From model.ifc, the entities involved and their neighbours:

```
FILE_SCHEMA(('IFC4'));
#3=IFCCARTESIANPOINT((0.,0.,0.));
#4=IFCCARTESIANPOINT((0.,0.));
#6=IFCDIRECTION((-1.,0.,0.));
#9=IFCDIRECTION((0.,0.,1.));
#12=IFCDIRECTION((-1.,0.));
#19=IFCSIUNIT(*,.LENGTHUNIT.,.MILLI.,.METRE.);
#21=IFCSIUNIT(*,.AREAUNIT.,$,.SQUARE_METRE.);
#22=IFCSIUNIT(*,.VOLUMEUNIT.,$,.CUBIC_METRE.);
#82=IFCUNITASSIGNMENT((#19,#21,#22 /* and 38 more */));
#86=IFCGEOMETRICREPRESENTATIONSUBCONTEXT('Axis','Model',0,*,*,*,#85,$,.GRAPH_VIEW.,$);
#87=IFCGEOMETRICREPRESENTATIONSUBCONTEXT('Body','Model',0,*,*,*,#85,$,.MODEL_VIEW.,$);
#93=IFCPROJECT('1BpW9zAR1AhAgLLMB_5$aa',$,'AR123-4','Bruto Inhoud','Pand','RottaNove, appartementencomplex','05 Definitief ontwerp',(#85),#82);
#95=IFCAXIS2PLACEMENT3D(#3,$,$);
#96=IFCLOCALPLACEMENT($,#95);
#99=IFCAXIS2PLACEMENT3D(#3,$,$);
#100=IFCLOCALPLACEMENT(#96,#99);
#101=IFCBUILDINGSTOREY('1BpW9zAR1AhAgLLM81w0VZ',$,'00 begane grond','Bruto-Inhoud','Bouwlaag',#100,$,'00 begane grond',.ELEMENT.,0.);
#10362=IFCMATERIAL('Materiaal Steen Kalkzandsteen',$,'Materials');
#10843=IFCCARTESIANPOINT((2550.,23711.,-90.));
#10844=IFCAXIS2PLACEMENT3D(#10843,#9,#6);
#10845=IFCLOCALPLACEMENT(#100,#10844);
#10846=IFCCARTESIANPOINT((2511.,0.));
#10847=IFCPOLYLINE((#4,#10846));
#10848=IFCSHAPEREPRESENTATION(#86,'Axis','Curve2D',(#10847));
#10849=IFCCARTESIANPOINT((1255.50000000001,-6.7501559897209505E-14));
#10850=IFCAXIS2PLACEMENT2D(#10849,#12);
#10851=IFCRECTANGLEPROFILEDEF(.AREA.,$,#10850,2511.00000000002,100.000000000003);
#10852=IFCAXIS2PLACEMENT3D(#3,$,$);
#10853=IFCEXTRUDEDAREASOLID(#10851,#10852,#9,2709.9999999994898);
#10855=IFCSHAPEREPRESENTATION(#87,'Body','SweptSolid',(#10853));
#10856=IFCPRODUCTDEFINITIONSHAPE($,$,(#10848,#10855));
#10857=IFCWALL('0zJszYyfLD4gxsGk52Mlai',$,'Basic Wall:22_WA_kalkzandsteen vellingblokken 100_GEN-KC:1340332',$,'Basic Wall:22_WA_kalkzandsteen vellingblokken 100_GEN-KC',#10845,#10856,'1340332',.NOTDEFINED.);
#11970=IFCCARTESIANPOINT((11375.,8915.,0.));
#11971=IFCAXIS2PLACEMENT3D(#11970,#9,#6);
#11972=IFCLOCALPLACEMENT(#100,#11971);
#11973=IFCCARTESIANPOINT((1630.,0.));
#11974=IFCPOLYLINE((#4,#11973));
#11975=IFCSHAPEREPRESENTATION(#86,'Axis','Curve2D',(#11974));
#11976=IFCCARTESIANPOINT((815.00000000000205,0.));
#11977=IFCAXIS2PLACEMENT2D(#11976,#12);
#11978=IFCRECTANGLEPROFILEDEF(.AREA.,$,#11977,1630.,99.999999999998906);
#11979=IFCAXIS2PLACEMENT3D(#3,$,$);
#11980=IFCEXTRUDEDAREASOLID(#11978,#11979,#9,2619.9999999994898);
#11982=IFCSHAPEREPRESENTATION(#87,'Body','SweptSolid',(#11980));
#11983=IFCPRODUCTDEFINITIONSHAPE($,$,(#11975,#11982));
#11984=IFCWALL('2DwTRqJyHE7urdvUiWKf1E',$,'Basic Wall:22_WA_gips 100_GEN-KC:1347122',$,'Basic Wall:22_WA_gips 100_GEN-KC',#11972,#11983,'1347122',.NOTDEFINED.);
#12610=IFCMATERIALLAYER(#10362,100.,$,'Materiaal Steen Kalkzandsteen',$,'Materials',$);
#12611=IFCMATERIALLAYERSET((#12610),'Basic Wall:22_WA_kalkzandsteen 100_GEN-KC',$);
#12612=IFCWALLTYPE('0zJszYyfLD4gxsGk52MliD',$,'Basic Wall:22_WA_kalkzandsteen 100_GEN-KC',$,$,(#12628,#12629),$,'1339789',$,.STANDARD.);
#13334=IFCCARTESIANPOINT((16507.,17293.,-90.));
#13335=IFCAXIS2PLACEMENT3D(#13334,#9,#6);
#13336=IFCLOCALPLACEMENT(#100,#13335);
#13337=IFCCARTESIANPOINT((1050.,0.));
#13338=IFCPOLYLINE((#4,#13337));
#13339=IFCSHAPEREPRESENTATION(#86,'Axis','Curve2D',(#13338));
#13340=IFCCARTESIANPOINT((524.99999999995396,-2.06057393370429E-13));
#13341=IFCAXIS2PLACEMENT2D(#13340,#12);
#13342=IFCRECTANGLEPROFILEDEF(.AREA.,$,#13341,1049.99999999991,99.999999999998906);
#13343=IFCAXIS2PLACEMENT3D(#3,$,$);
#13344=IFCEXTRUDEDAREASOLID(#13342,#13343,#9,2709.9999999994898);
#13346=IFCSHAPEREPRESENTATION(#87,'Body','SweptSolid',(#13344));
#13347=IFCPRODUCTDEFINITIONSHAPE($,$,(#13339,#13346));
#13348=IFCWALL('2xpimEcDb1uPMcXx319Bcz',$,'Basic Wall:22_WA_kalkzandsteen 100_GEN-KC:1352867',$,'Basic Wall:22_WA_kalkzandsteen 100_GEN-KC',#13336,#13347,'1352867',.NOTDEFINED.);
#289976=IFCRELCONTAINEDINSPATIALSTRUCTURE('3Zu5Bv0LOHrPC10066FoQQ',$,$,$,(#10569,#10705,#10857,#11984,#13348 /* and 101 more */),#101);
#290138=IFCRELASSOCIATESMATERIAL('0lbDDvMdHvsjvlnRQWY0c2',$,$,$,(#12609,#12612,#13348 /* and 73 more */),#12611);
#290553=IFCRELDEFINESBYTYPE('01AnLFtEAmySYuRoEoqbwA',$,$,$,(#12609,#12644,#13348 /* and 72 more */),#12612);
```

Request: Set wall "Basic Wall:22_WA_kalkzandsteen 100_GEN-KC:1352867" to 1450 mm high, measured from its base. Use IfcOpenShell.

```python
import ifcopenshell
import ifcopenshell.geom
import ifcopenshell.util.representation
import ifcopenshell.util.shape

model = ifcopenshell.open("model.ifc")
settings = ifcopenshell.geom.settings()


def volume(element):
    """Net volume in cubic metres, openings subtracted."""
    shape = ifcopenshell.geom.create_shape(settings, element)
    return ifcopenshell.util.shape.get_volume(shape.geometry)


wall = model.by_id(13348)
before = volume(wall)

body = ifcopenshell.util.representation.get_representation(wall, "Model", "Body")
solid = body.Items[0]
old_height = solid.Depth
solid.Depth = 1450.0
after = volume(wall)

print(f"height {old_height:g} -> {solid.Depth:g}, volume {before:.3f} -> {after:.3f} m3")

model.write("model_edited.ifc")
```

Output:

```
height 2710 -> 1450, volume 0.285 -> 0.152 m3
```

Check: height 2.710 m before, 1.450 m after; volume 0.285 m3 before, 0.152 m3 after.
